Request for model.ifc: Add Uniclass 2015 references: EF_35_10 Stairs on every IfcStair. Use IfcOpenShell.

First a look at what the model holds.

```python
import ifcopenshell

model = ifcopenshell.open("model.ifc")
print(model.schema)
print("classifications:", [c.Name for c in model.by_type("IfcClassification")])
for ifc_class in ("IfcDoor", "IfcRoof", "IfcStair", "IfcWall", "IfcWindow"):
    print(ifc_class, len(model.by_type(ifc_class)))
```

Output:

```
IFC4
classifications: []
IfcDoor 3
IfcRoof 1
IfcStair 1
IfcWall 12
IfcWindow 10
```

```python
import ifcopenshell
import ifcopenshell.api.classification

model = ifcopenshell.open("model.ifc")

system = ifcopenshell.api.classification.add_classification(model, classification="Uniclass 2015")

codes = {
    "IfcStair": ("EF_35_10", "Stairs"),
}
for ifc_class, (code, name) in codes.items():
    products = model.by_type(ifc_class)
    ifcopenshell.api.classification.add_reference(
        model, products=products, classification=system, identification=code, name=name
    )
    print(code, len(products))

model.write("model_updated.ifc")
```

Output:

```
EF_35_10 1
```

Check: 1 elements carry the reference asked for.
